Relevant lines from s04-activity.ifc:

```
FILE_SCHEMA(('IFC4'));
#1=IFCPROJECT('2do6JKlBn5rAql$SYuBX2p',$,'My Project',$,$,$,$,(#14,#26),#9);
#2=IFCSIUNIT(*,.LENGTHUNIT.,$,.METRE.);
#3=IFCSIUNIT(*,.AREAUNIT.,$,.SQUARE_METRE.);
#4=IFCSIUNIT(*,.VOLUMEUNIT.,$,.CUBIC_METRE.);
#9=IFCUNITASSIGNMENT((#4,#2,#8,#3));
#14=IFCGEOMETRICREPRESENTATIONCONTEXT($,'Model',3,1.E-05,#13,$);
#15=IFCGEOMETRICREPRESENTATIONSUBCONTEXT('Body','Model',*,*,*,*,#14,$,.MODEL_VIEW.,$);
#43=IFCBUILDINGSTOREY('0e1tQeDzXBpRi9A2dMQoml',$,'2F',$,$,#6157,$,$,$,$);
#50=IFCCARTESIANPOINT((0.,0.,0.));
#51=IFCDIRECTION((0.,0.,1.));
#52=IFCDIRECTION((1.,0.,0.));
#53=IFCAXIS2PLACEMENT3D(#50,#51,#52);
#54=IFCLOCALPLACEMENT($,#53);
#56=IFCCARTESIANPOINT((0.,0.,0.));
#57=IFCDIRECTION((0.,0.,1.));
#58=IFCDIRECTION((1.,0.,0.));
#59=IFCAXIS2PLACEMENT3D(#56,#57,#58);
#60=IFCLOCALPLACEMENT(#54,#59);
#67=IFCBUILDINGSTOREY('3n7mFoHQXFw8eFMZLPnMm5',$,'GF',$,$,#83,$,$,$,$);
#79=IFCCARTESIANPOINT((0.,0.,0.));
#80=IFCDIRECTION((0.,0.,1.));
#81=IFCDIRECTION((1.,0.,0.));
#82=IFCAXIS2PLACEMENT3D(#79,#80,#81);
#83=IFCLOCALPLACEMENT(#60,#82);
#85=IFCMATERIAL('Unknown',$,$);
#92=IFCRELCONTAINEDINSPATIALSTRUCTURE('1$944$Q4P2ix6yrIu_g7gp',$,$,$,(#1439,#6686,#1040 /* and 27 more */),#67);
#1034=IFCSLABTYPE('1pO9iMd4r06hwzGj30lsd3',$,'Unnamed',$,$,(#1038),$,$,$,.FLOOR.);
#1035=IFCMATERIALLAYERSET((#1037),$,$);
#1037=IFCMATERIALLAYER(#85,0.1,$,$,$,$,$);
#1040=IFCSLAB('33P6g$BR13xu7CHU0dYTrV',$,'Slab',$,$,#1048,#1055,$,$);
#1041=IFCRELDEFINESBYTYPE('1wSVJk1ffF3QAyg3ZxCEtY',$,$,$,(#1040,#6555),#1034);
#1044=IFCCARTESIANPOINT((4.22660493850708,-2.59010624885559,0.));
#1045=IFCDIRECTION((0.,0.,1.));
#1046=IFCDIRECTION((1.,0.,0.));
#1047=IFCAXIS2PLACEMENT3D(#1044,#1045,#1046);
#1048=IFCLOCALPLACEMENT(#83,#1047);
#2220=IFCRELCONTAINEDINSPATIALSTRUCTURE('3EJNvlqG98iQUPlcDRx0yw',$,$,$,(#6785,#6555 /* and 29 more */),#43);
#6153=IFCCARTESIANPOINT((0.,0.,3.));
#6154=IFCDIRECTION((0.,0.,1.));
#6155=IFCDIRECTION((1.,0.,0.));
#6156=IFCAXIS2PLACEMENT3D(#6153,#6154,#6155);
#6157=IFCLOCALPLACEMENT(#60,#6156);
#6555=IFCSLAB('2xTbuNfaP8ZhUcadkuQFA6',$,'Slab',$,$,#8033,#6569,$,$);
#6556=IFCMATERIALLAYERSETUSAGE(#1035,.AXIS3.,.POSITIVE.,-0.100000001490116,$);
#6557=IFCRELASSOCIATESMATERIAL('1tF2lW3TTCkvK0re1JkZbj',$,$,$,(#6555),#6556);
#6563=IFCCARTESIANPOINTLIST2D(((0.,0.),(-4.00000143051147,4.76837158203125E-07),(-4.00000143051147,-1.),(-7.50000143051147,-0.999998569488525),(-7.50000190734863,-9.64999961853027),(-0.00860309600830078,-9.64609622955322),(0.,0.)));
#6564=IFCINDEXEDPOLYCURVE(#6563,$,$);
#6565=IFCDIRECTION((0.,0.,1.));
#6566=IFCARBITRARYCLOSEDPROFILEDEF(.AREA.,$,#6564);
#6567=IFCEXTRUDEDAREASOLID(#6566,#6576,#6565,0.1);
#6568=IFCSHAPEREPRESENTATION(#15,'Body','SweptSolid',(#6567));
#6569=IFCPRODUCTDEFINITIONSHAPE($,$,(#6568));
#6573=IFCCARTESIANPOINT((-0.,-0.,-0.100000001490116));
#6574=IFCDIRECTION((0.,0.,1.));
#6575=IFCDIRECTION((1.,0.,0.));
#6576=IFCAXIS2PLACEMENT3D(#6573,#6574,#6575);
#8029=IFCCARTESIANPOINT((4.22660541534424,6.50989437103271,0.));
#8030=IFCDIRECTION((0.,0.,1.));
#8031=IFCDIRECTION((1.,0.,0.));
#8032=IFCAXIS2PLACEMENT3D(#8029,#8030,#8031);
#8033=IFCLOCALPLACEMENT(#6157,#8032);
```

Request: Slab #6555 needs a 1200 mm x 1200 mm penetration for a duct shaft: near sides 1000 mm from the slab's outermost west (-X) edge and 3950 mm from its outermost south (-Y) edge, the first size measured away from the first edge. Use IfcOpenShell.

```python
import numpy as np
import ifcopenshell
import ifcopenshell.api.feature
import ifcopenshell.api.geometry
import ifcopenshell.api.root
import ifcopenshell.geom
import ifcopenshell.util.placement
import ifcopenshell.util.representation
import ifcopenshell.util.shape
import ifcopenshell.util.unit

model = ifcopenshell.open("s04-activity.ifc")
unit_scale = ifcopenshell.util.unit.calculate_unit_scale(model)
settings = ifcopenshell.geom.settings()


def volume(element):
    """Net volume in cubic metres, openings subtracted."""
    shape = ifcopenshell.geom.create_shape(settings, element)
    return ifcopenshell.util.shape.get_volume(shape.geometry)


slab = model.by_guid("2xTbuNfaP8ZhUcadkuQFA6")
before = volume(slab)

# Extent in the slab's own axes, in metres. The edges named are its -X and -Y sides.
slab_shape = ifcopenshell.geom.create_shape(settings, slab)
vertices = ifcopenshell.util.shape.get_vertices(slab_shape.geometry)
x_min, y_min, bottom = vertices.min(axis=0)
top = vertices[:, 2].max()

opening = ifcopenshell.api.root.create_entity(model, ifc_class="IfcOpeningElement", name="Duct shaft opening", predefined_type="OPENING")
context = ifcopenshell.util.representation.get_context(model, "Model", "Body", "MODEL_VIEW")
width, depth = 1.2, 1.2
outline = [(0.0, 0.0), (width, 0.0), (width, depth), (0.0, depth), (0.0, 0.0)]
# Overshoot both faces by 50 mm so the cut is clean.
shape = ifcopenshell.api.geometry.add_slab_representation(
    model, context=context, depth=top - bottom + 0.1, polyline=outline
)
ifcopenshell.api.geometry.assign_representation(model, product=opening, representation=shape)

matrix = ifcopenshell.util.placement.get_local_placement(slab.ObjectPlacement)
matrix[:, 3] = matrix @ np.append(np.array([x_min + 1, y_min + 3.95, bottom - 0.05]) / unit_scale, 1.0)
ifcopenshell.api.geometry.edit_object_placement(model, product=opening, matrix=matrix, is_si=False)
ifcopenshell.api.feature.add_feature(model, feature=opening, element=slab)

after = volume(slab)

print(f"slab volume {before:.3f} -> {after:.3f} m3")

model.write("s04-activity_v2.ifc")
```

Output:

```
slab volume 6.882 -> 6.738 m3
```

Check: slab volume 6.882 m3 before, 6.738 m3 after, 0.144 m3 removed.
